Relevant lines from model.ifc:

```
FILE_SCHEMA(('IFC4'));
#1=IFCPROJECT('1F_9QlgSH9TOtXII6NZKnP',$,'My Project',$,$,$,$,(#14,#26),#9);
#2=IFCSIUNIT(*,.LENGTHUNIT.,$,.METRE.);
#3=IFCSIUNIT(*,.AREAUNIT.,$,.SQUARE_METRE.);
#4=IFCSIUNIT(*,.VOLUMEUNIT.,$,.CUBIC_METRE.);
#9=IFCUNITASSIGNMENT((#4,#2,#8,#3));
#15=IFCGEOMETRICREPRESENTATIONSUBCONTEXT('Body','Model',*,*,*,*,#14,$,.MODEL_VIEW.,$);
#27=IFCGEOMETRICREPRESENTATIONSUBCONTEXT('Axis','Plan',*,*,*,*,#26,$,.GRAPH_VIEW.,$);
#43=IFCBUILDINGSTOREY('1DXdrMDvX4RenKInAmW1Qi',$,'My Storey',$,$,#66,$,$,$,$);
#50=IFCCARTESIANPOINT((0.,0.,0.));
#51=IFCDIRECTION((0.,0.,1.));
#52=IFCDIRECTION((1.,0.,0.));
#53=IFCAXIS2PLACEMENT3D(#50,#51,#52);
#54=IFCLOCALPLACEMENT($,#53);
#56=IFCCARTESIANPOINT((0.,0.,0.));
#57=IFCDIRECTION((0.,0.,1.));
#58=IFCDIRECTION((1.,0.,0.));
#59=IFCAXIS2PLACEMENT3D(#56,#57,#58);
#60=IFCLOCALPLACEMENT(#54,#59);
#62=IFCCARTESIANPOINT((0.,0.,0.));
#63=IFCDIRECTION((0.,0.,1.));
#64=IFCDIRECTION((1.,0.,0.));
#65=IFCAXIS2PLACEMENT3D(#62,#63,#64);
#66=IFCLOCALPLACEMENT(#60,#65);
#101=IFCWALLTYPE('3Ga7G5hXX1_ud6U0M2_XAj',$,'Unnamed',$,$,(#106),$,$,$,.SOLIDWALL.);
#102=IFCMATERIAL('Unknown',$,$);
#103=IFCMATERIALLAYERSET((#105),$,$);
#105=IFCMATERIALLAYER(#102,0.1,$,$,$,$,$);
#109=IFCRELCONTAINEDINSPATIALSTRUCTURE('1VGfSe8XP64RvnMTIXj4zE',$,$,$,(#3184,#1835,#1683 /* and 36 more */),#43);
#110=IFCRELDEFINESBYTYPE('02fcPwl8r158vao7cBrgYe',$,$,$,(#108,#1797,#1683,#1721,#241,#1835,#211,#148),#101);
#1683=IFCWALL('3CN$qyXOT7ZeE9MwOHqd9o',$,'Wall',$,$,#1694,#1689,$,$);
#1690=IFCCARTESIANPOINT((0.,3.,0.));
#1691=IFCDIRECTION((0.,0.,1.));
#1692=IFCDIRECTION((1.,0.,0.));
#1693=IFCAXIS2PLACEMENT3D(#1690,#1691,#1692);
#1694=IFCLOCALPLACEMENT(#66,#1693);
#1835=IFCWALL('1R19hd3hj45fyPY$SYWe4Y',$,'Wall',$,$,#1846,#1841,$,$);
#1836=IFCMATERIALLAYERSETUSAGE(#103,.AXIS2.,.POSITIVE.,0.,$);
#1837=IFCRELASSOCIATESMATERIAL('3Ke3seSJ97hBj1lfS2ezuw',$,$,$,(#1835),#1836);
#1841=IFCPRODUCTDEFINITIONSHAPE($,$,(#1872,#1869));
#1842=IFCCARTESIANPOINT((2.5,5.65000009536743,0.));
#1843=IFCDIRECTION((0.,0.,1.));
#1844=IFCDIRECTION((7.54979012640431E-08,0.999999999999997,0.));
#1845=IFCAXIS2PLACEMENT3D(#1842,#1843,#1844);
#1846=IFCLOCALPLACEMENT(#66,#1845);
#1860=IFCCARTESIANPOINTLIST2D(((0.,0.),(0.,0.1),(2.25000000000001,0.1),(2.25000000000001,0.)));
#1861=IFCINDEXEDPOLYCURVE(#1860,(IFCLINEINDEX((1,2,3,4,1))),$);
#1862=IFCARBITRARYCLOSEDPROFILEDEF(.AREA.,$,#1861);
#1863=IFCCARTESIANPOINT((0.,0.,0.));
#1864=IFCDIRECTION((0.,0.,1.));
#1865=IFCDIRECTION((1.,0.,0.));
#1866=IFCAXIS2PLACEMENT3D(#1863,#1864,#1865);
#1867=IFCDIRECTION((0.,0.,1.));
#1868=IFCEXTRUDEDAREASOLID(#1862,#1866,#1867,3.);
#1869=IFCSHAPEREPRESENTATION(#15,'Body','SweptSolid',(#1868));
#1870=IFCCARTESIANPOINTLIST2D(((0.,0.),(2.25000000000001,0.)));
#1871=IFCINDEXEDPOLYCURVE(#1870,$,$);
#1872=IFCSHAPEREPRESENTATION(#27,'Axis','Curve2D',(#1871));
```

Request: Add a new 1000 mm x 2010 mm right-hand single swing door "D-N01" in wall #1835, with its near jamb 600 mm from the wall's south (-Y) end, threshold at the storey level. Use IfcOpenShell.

```python
import numpy as np
import ifcopenshell
import ifcopenshell.api.feature
import ifcopenshell.api.geometry
import ifcopenshell.api.root
import ifcopenshell.api.spatial
import ifcopenshell.geom
import ifcopenshell.util.element
import ifcopenshell.util.placement
import ifcopenshell.util.representation
import ifcopenshell.util.shape
import ifcopenshell.util.unit

model = ifcopenshell.open("model.ifc")
unit_scale = ifcopenshell.util.unit.calculate_unit_scale(model)
settings = ifcopenshell.geom.settings()


def volume(element):
    """Net volume in cubic metres, openings subtracted."""
    shape = ifcopenshell.geom.create_shape(settings, element)
    return ifcopenshell.util.shape.get_volume(shape.geometry)


wall = model.by_id(1835)
storey = ifcopenshell.util.element.get_container(wall, ifc_class="IfcBuildingStorey")
context = ifcopenshell.util.representation.get_context(model, "Model", "Body", "MODEL_VIEW")
before = volume(wall)

width, height, from_end, sill = 1, 2.01, 0.6, 0.0  # metres

# The wall runs along its own X axis, and the end named is its -X end.
wall_shape = ifcopenshell.geom.create_shape(settings, wall)
x, y, z = ifcopenshell.util.shape.get_vertices(wall_shape.geometry).T
start = x.min() + from_end
face, thickness = float(y.min()), float(y.max() - y.min())
wall_matrix = ifcopenshell.util.placement.get_local_placement(wall.ObjectPlacement)
level = ifcopenshell.util.placement.get_local_placement(storey.ObjectPlacement)[2, 3]


def in_wall(x, y):
    """Placement at x, y metres in the wall's axes, at sill height."""
    matrix = wall_matrix.copy()
    matrix[:, 3] = wall_matrix @ np.array([x / unit_scale, y / unit_scale, 0.0, 1.0])
    matrix[2, 3] = level + sill / unit_scale
    return matrix


# Opening: a box that overshoots both wall faces by 50 mm.
opening = ifcopenshell.api.root.create_entity(model, ifc_class="IfcOpeningElement", predefined_type="OPENING")
box = ifcopenshell.api.geometry.add_wall_representation(
    model, context=context, length=width, height=height, thickness=thickness + 0.1
)
ifcopenshell.api.geometry.assign_representation(model, product=opening, representation=box)
ifcopenshell.api.geometry.edit_object_placement(model, product=opening, matrix=in_wall(start, face - 0.05), is_si=False)
ifcopenshell.api.feature.add_feature(model, feature=opening, element=wall)

door = ifcopenshell.api.root.create_entity(model, ifc_class="IfcDoor", name="D-N01", predefined_type="DOOR")
door.OverallWidth, door.OverallHeight = width / unit_scale, height / unit_scale
door.OperationType = "SINGLE_SWING_RIGHT"
body = ifcopenshell.api.geometry.add_door_representation(
    model,
    context=context,
    overall_width=door.OverallWidth,
    overall_height=door.OverallHeight,
    operation_type="SINGLE_SWING_RIGHT",
    lining_properties={"LiningDepth": thickness / unit_scale, "ThresholdDepth": thickness / unit_scale},
)
ifcopenshell.api.geometry.assign_representation(model, product=door, representation=body)
ifcopenshell.api.spatial.assign_container(model, products=[door], relating_structure=storey)
ifcopenshell.api.feature.add_filling(model, opening=opening, element=door)

# The lining spans the wall, so the door starts at the wall face.
ifcopenshell.api.geometry.edit_object_placement(model, product=door, matrix=in_wall(start, face), is_si=False)

after = volume(wall)

print(f"wall volume {before:.3f} -> {after:.3f} m3")

model.write("model_rev.ifc")
```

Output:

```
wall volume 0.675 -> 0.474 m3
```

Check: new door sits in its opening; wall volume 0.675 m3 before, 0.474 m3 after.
